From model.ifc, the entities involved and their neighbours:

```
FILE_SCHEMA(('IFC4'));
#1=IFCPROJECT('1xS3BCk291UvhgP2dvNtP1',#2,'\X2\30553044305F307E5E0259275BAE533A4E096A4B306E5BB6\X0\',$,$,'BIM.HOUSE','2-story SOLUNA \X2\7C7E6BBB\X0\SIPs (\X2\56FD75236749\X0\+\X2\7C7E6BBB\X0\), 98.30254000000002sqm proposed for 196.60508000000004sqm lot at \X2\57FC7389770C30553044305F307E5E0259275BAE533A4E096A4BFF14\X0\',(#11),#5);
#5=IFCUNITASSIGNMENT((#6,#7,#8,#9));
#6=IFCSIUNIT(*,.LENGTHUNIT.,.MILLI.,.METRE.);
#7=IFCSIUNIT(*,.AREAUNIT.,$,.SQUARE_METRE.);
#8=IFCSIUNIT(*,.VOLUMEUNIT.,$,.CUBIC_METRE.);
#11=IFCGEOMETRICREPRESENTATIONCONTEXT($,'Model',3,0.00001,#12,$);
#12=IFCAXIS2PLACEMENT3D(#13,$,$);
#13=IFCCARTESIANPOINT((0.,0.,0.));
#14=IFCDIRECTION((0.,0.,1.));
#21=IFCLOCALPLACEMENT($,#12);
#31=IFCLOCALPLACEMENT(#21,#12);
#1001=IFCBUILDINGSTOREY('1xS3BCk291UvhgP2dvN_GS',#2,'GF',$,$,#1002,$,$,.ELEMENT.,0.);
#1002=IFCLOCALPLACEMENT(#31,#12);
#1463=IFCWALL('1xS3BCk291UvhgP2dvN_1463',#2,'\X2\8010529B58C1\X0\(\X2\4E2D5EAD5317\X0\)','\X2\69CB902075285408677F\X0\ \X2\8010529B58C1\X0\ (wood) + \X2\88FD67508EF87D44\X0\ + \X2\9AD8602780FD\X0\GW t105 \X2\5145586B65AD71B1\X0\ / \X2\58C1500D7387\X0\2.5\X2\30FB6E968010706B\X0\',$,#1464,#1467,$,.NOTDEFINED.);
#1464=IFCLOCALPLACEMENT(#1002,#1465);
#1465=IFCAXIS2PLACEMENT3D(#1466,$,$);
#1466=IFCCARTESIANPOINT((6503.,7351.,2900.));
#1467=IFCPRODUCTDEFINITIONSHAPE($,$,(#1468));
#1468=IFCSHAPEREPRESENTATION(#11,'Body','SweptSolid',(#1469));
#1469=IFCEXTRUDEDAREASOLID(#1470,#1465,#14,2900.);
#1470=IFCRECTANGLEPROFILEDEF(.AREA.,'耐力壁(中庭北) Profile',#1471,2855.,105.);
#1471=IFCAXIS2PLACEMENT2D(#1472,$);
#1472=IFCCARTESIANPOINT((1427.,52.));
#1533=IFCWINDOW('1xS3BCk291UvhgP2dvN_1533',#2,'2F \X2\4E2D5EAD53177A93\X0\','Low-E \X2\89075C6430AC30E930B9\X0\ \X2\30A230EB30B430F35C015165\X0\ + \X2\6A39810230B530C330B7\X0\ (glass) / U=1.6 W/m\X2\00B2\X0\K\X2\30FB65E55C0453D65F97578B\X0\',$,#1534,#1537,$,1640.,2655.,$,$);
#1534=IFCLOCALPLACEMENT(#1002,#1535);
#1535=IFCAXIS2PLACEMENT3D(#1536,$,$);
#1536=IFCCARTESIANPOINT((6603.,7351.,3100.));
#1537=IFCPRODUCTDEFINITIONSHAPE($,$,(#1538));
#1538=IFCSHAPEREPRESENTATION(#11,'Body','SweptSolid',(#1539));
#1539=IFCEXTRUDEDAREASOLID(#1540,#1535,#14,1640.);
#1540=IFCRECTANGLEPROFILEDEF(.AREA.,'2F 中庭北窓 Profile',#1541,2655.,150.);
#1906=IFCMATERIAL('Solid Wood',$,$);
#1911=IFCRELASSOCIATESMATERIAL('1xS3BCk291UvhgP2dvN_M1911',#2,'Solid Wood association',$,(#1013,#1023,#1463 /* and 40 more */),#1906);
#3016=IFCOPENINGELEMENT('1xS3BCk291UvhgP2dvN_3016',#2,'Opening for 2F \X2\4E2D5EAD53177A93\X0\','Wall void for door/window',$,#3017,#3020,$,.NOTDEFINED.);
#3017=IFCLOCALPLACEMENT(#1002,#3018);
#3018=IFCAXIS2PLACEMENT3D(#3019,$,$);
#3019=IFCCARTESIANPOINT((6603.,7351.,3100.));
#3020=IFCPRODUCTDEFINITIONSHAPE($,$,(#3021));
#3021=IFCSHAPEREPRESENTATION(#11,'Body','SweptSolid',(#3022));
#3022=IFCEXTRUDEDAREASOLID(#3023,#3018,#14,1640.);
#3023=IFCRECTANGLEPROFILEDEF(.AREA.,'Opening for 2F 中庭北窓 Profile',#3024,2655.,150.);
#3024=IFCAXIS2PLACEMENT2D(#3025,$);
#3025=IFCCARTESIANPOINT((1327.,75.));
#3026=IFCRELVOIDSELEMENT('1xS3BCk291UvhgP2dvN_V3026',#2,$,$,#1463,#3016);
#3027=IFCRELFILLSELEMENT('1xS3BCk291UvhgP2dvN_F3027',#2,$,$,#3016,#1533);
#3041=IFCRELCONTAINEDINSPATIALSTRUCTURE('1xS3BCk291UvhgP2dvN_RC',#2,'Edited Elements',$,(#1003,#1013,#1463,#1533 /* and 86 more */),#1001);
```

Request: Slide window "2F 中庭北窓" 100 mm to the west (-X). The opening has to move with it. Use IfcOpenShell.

```python
import ifcopenshell
import ifcopenshell.api.geometry
import ifcopenshell.util.placement

model = ifcopenshell.open("model.ifc")

window = model.by_guid("1xS3BCk291UvhgP2dvN_1533")
opening = window.FillsVoids[0].RelatingOpeningElement
wall = opening.VoidsElements[0].RelatingBuildingElement

wall_matrix = ifcopenshell.util.placement.get_local_placement(wall.ObjectPlacement)
shift = wall_matrix[:3, 0] * -100.0
before = ifcopenshell.util.placement.get_local_placement(window.ObjectPlacement)[:3, 3].copy()

# The window is not placed relative to its opening, so move both.
for product in (opening, window):
    matrix = ifcopenshell.util.placement.get_local_placement(product.ObjectPlacement)
    matrix[:3, 3] += shift
    ifcopenshell.api.geometry.edit_object_placement(model, product=product, matrix=matrix, is_si=False)

after = ifcopenshell.util.placement.get_local_placement(window.ObjectPlacement)[:3, 3]
print("window moved by", (after - before).round(3) + 0.0)

model.write("model_rev.ifc")
```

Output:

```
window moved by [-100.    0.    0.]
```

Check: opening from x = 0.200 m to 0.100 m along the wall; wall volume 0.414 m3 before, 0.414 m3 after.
